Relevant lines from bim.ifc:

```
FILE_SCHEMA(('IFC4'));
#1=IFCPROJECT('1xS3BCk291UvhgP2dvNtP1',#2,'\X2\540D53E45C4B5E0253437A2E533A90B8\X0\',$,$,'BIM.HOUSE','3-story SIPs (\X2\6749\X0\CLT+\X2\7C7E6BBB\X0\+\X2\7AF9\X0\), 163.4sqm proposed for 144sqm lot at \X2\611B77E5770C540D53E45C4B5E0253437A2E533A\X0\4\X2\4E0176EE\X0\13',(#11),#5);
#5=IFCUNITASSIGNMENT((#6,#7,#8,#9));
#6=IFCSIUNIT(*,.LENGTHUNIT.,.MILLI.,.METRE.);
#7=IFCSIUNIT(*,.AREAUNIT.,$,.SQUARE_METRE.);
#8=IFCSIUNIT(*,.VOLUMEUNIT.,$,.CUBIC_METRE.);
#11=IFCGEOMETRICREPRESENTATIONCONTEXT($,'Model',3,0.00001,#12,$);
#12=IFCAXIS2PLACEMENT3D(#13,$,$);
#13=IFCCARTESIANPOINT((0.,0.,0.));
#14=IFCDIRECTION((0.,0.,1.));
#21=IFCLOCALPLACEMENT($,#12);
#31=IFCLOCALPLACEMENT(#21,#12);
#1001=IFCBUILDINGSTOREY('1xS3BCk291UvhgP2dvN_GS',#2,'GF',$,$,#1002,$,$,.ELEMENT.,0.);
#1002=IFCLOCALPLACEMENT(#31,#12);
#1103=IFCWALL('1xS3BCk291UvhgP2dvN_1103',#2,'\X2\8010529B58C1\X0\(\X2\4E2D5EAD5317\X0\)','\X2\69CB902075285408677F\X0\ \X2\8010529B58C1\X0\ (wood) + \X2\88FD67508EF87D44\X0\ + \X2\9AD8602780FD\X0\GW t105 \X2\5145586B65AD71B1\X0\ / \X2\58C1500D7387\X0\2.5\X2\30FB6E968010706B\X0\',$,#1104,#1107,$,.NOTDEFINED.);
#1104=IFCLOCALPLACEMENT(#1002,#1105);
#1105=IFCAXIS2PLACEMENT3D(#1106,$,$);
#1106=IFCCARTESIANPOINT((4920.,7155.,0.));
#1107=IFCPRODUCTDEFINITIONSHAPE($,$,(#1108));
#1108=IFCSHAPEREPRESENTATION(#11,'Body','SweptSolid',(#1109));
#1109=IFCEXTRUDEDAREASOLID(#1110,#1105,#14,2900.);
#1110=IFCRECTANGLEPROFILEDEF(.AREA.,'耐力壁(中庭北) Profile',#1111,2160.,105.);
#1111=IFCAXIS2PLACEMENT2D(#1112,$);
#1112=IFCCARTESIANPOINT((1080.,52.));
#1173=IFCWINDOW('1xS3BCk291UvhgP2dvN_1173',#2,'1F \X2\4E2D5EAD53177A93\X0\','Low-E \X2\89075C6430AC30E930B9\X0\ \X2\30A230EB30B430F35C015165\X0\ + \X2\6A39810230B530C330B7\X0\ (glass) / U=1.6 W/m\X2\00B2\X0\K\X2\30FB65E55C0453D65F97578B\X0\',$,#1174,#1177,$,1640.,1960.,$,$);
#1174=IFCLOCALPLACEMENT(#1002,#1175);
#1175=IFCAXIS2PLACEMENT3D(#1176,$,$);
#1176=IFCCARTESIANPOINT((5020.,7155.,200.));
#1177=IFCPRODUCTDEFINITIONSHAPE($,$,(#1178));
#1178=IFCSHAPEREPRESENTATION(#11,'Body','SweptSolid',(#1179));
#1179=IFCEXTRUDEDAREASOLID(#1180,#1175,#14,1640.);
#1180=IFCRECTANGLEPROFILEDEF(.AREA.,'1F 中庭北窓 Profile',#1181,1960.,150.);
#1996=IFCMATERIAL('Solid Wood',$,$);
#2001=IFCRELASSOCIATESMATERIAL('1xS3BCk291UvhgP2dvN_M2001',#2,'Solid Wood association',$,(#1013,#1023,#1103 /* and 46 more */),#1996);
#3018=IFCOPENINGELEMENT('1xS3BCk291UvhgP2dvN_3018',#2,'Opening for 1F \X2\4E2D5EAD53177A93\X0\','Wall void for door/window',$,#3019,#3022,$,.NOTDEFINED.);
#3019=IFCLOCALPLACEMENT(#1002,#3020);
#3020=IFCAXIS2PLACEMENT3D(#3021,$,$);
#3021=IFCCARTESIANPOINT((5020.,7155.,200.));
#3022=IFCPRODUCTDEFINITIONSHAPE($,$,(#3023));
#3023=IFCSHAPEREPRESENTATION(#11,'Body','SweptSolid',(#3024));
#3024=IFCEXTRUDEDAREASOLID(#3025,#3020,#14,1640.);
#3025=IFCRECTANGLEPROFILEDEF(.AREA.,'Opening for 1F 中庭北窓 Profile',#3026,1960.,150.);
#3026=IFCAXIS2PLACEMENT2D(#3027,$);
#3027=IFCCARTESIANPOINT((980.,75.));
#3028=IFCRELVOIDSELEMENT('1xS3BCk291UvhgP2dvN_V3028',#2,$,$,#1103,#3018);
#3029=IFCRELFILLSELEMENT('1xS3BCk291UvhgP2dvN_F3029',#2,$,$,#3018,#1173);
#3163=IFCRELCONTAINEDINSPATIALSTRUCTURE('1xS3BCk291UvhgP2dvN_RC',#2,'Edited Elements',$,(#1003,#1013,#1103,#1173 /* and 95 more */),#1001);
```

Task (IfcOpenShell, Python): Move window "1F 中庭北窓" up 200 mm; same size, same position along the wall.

```python
import numpy as np
import ifcopenshell
import ifcopenshell.api.geometry
import ifcopenshell.util.placement
import ifcopenshell.util.unit

model = ifcopenshell.open("bim.ifc")
unit_scale = ifcopenshell.util.unit.calculate_unit_scale(model)

window = model.by_guid("1xS3BCk291UvhgP2dvN_1173")
opening = window.FillsVoids[0].RelatingOpeningElement
dz = 200.0

shift = np.array([0.0, 0.0, dz])
# The window is not placed relative to its opening, so move both.
for product in (opening, window):
    matrix = ifcopenshell.util.placement.get_local_placement(product.ObjectPlacement)
    matrix[:3, 3] += shift
    ifcopenshell.api.geometry.edit_object_placement(model, product=product, matrix=matrix, is_si=False)

print(f"moved by {dz * unit_scale:+.3f} m")

model.write("bim_updated.ifc")
```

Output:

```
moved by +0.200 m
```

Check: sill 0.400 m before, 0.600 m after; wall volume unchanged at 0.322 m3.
